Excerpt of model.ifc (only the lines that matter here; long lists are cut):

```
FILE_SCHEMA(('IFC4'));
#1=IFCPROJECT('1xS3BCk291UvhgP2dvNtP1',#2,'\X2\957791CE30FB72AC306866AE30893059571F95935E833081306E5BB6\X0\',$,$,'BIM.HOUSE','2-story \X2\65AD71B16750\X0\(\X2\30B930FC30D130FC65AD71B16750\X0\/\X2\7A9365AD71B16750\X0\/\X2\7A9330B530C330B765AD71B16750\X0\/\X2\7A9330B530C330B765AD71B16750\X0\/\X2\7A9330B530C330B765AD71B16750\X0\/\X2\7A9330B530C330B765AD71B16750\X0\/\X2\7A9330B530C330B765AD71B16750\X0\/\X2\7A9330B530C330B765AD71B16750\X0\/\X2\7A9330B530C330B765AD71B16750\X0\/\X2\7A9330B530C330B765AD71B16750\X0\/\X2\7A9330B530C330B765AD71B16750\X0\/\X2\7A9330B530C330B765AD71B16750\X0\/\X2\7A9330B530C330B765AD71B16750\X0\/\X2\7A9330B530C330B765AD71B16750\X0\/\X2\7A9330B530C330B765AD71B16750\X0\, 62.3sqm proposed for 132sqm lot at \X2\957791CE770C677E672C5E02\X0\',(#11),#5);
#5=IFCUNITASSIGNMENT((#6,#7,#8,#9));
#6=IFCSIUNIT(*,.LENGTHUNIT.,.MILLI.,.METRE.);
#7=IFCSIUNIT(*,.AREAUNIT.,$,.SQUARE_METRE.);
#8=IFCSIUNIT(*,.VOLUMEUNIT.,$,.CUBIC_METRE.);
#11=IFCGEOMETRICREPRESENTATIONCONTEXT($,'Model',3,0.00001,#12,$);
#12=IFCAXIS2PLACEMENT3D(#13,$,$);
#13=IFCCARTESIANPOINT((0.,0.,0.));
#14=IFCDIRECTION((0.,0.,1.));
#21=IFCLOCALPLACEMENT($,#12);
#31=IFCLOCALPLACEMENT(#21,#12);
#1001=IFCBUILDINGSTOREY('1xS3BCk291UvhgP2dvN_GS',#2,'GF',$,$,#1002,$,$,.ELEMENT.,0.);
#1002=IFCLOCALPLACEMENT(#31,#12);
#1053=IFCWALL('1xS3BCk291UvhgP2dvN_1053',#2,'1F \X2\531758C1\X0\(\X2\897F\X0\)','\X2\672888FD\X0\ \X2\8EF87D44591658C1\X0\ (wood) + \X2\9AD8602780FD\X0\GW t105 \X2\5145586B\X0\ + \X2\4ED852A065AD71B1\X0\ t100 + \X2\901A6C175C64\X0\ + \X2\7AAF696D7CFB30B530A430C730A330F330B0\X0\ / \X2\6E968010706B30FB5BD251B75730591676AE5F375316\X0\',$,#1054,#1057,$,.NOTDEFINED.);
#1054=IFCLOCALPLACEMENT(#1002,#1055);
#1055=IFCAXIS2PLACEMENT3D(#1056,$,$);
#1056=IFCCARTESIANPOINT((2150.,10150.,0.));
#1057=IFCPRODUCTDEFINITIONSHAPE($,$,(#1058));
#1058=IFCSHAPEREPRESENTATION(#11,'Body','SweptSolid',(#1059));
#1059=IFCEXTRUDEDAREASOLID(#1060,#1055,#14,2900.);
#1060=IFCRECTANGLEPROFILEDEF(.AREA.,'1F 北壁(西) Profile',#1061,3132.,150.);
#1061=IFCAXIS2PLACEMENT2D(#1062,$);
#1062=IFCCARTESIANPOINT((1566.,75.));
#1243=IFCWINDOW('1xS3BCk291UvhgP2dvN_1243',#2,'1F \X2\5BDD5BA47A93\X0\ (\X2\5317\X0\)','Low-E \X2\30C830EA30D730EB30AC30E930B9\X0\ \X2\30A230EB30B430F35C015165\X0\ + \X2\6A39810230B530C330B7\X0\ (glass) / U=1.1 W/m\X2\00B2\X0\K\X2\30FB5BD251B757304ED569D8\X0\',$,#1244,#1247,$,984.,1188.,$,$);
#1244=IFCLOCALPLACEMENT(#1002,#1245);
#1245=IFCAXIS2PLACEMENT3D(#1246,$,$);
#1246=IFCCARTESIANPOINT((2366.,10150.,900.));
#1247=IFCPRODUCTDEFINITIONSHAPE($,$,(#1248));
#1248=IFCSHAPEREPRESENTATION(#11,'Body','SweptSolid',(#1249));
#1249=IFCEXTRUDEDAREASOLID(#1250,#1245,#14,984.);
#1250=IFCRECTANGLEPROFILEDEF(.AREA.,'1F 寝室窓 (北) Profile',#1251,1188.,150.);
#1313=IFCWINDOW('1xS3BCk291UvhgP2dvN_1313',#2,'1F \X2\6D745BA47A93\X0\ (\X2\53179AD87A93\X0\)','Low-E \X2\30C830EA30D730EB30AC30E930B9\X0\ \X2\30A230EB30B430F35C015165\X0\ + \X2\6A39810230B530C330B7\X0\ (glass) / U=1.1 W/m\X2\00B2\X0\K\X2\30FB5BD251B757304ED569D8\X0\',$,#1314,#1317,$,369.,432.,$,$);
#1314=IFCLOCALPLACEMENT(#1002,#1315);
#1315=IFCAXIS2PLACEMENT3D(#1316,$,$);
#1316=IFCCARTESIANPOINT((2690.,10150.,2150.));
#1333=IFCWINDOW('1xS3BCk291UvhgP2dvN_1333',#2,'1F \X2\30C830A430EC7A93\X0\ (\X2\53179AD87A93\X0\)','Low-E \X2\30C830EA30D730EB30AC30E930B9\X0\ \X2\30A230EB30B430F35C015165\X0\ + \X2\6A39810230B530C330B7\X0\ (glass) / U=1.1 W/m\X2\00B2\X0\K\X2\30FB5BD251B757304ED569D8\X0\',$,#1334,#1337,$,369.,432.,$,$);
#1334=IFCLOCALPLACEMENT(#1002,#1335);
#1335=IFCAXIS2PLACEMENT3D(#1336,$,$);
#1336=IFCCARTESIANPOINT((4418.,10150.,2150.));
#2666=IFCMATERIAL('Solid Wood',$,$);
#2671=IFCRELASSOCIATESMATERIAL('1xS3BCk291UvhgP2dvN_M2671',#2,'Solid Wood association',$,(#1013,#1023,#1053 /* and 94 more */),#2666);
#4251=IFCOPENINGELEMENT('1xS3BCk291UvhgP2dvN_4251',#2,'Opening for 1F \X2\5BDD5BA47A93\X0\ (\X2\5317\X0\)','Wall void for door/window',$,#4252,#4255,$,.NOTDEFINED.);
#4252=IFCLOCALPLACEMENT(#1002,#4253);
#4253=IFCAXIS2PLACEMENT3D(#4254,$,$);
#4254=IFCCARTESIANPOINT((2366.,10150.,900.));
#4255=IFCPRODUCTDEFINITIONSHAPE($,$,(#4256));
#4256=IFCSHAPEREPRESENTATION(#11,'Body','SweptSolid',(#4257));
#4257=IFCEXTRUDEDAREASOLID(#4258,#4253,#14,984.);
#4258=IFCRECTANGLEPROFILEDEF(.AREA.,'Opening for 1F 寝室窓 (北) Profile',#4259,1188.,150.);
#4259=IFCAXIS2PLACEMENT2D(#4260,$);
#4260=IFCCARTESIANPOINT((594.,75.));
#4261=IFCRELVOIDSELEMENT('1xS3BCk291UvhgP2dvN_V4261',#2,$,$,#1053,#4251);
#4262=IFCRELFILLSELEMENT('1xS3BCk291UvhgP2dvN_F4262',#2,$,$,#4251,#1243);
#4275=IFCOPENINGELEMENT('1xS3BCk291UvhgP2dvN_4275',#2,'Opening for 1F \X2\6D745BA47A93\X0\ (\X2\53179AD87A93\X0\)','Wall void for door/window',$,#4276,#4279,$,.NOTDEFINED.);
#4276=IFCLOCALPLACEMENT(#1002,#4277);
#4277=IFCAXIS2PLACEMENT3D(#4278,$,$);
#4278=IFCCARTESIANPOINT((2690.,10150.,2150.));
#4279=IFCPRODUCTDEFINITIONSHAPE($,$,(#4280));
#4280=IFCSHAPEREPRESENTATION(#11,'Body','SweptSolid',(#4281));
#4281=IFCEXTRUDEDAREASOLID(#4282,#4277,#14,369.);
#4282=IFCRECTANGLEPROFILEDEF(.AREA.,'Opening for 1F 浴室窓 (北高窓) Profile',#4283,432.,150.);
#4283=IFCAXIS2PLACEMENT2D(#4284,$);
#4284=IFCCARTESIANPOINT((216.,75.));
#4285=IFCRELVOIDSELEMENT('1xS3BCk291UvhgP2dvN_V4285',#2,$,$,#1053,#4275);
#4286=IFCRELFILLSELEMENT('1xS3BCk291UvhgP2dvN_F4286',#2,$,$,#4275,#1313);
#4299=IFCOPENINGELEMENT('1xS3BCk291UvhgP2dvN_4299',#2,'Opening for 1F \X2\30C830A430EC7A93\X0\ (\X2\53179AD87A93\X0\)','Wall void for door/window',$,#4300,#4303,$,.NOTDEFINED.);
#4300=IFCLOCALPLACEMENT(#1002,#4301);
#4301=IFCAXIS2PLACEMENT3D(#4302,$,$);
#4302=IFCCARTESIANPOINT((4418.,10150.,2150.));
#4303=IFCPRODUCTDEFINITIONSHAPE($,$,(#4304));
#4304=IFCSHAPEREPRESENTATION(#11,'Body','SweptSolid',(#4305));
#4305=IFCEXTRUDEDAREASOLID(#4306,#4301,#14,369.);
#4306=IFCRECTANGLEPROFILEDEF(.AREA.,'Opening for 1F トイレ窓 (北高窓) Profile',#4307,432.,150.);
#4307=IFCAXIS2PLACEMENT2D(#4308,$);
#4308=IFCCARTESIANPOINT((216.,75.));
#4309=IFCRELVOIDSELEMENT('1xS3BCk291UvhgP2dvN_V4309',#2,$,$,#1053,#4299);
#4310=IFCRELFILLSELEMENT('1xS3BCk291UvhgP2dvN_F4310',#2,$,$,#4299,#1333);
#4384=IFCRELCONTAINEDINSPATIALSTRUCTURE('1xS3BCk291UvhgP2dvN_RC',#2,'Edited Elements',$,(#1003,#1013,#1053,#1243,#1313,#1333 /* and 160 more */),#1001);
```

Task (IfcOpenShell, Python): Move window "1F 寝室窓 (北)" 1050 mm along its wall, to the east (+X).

```python
import ifcopenshell
import ifcopenshell.api.geometry
import ifcopenshell.util.placement

model = ifcopenshell.open("model.ifc")

window = model.by_guid("1xS3BCk291UvhgP2dvN_1243")
opening = window.FillsVoids[0].RelatingOpeningElement
wall = opening.VoidsElements[0].RelatingBuildingElement

wall_matrix = ifcopenshell.util.placement.get_local_placement(wall.ObjectPlacement)
shift = wall_matrix[:3, 0] * 1050.0
before = ifcopenshell.util.placement.get_local_placement(window.ObjectPlacement)[:3, 3].copy()

# The window is not placed relative to its opening, so move both.
for product in (opening, window):
    matrix = ifcopenshell.util.placement.get_local_placement(product.ObjectPlacement)
    matrix[:3, 3] += shift
    ifcopenshell.api.geometry.edit_object_placement(model, product=product, matrix=matrix, is_si=False)

after = ifcopenshell.util.placement.get_local_placement(window.ObjectPlacement)[:3, 3]
print("window moved by", (after - before).round(3) + 0.0)

model.write("model_edited.ifc")
```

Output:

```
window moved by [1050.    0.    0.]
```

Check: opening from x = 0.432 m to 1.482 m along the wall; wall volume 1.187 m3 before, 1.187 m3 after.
